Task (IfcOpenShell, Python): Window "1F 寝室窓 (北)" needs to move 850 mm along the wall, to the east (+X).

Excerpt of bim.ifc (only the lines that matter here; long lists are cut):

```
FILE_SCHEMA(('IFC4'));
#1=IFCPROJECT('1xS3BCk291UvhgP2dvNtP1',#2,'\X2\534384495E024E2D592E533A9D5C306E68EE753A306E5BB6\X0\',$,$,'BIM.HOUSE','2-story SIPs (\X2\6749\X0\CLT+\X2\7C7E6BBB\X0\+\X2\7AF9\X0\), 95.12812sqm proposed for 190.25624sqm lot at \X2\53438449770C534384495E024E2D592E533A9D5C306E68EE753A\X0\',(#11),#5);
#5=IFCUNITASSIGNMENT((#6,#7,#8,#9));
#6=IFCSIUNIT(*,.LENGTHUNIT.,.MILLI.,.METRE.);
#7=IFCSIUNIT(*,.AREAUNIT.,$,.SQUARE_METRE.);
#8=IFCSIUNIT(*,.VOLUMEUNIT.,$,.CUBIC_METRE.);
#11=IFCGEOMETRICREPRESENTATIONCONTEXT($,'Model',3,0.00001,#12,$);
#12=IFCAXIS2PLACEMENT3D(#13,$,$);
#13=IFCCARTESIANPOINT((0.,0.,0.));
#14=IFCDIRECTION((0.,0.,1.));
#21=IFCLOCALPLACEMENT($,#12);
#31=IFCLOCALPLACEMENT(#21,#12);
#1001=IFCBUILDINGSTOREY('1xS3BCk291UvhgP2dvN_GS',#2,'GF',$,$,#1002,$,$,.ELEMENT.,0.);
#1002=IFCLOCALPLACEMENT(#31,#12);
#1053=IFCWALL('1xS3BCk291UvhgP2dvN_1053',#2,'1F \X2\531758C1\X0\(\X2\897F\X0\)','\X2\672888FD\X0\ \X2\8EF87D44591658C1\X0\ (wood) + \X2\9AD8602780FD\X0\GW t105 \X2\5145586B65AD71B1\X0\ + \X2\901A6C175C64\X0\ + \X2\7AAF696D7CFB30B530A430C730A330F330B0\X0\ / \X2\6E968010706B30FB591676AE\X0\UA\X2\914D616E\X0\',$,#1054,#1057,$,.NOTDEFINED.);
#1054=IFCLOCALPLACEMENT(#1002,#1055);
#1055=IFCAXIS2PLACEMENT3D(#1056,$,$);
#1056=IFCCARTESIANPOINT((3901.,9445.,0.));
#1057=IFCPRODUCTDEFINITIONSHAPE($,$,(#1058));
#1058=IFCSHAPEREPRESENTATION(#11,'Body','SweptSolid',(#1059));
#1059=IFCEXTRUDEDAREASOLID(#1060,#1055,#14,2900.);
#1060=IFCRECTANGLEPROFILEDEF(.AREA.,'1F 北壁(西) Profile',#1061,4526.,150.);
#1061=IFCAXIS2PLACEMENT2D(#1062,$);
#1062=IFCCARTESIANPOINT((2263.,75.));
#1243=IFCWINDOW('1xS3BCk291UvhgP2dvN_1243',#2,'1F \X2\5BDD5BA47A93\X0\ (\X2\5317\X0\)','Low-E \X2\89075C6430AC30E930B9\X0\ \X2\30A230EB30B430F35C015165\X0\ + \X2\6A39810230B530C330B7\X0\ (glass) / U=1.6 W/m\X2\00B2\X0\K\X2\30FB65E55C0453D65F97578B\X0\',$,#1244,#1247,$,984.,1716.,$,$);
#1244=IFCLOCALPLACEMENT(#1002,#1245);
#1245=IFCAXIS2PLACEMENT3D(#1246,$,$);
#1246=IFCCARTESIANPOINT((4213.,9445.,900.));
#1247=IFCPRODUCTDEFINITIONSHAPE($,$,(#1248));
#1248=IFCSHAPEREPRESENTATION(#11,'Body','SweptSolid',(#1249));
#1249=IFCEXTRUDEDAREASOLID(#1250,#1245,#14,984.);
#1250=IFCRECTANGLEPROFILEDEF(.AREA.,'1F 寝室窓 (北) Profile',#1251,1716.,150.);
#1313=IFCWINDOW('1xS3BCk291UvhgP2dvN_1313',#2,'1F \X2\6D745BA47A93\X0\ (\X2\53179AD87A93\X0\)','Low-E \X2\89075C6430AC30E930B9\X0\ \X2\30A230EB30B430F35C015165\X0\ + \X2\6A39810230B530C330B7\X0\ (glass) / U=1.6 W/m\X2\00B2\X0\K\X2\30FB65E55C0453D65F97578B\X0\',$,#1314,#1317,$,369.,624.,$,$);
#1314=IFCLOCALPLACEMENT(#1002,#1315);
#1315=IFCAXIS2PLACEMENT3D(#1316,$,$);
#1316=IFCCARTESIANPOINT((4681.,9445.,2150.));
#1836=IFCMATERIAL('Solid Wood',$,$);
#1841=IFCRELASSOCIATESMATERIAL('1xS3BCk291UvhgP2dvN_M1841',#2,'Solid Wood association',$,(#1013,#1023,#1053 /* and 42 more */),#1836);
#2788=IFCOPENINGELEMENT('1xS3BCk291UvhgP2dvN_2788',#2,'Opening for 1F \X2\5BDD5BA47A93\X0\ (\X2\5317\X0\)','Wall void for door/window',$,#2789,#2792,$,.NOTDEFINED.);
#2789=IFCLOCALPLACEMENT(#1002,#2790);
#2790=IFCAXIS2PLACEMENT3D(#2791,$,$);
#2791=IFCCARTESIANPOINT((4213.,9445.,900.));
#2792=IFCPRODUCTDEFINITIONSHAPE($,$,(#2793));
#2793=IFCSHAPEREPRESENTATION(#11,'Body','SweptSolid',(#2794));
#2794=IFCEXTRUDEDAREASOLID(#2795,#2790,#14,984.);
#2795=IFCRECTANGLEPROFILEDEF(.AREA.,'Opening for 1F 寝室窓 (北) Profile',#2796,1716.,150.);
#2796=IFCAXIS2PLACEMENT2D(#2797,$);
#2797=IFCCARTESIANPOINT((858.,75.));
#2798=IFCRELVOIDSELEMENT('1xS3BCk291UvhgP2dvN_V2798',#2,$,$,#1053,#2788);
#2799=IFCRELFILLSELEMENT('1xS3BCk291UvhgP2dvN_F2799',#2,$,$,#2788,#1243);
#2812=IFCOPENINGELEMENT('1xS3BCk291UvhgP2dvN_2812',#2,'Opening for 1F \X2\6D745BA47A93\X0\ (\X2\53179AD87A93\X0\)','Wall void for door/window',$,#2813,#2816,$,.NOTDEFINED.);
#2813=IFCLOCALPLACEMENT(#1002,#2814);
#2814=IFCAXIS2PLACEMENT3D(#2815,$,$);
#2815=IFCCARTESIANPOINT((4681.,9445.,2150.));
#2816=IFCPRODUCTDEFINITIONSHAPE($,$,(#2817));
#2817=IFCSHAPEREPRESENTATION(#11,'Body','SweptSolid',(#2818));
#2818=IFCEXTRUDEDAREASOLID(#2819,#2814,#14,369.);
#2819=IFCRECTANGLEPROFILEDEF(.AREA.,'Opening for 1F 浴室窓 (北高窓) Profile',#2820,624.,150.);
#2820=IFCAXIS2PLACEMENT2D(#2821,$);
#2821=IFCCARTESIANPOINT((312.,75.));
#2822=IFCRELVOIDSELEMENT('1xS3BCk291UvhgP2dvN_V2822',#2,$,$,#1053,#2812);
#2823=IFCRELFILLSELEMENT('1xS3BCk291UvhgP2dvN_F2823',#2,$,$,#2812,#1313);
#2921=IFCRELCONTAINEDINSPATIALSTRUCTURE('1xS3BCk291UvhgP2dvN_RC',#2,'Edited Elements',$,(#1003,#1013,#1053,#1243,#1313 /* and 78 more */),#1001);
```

```python
import ifcopenshell
import ifcopenshell.api.geometry
import ifcopenshell.util.placement
import ifcopenshell.util.unit

model = ifcopenshell.open("bim.ifc")
unit_scale = ifcopenshell.util.unit.calculate_unit_scale(model)

window = model.by_guid("1xS3BCk291UvhgP2dvN_1243")
opening = window.FillsVoids[0].RelatingOpeningElement
wall = opening.VoidsElements[0].RelatingBuildingElement

wall_matrix = ifcopenshell.util.placement.get_local_placement(wall.ObjectPlacement)
shift = wall_matrix[:3, 0] * 0.85 / unit_scale
before = ifcopenshell.util.placement.get_local_placement(window.ObjectPlacement)[:3, 3].copy()

# The window is not placed relative to its opening, so move both.
for product in (opening, window):
    matrix = ifcopenshell.util.placement.get_local_placement(product.ObjectPlacement)
    matrix[:3, 3] += shift
    ifcopenshell.api.geometry.edit_object_placement(model, product=product, matrix=matrix, is_si=False)

after = ifcopenshell.util.placement.get_local_placement(window.ObjectPlacement)[:3, 3]
print("window moved by", (after - before).round(3) + 0.0)

model.write("bim_edited.ifc")
```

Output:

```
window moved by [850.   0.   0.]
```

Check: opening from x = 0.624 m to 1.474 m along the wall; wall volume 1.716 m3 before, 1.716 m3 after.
